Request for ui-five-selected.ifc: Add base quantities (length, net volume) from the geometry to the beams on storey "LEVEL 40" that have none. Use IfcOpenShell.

First a look at what the model holds.

```python
import ifcopenshell
import ifcopenshell.util.element
import ifcopenshell.util.unit

model = ifcopenshell.open("ui-five-selected.ifc")
print(model.schema)
for unit_type in ("LENGTHUNIT", "AREAUNIT", "VOLUMEUNIT"):
    print(unit_type, ifcopenshell.util.unit.calculate_unit_scale(model, unit_type))
storey = next(s for s in model.by_type("IfcBuildingStorey") if s.Name == "LEVEL 40")
beams = [e for e in ifcopenshell.util.element.get_decomposition(storey) if e.is_a("IfcBeam")]
for e in sorted(beams, key=lambda e: e.id()):
    print(e.id(), e.is_a(), e.Name, list(ifcopenshell.util.element.get_psets(e, qtos_only=True)), sep=" | ")
```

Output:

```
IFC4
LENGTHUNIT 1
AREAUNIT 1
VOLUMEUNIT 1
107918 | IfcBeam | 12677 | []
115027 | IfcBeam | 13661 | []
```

```python
import ifcopenshell
import ifcopenshell.api.pset
import ifcopenshell.geom
import ifcopenshell.util.element
import ifcopenshell.util.shape
import ifcopenshell.util.unit

model = ifcopenshell.open("ui-five-selected.ifc")
unit_scale = ifcopenshell.util.unit.calculate_unit_scale(model)
volume_scale = ifcopenshell.util.unit.calculate_unit_scale(model, "VOLUMEUNIT")
settings = ifcopenshell.geom.settings()

storey = next(s for s in model.by_type("IfcBuildingStorey") if s.Name == "LEVEL 40")
beams = [e for e in ifcopenshell.util.element.get_decomposition(storey) if e.is_a("IfcBeam")]

for e in sorted(beams, key=lambda e: e.id()):
    if ifcopenshell.util.element.get_psets(e, qtos_only=True, should_inherit=False):
        continue
    # Geometry comes back in metres, in the element's own axes.
    shape = ifcopenshell.geom.create_shape(settings, e)
    values = {
        "Length": ifcopenshell.util.shape.get_max_xyz(shape.geometry) / unit_scale,
        "NetVolume": ifcopenshell.util.shape.get_volume(shape.geometry) / volume_scale,
    }
    qto = ifcopenshell.api.pset.add_qto(model, product=e, name="Qto_BeamBaseQuantities")
    ifcopenshell.api.pset.edit_qto(model, qto=qto, properties=values)
    print(e.id(), {k: round(v, 3) for k, v in values.items()})

model.write("ui-five-selected_updated.ifc")
```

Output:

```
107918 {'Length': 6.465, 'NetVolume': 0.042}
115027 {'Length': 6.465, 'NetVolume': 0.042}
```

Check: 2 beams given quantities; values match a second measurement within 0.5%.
